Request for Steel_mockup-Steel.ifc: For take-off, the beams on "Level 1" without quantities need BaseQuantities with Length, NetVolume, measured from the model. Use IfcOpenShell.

First a look at what the model holds.

```python
import ifcopenshell
import ifcopenshell.util.element
import ifcopenshell.util.unit

model = ifcopenshell.open("Steel_mockup-Steel.ifc")
print(model.schema)
for unit_type in ("LENGTHUNIT", "AREAUNIT", "VOLUMEUNIT"):
    print(unit_type, ifcopenshell.util.unit.calculate_unit_scale(model, unit_type))
storey = next(s for s in model.by_type("IfcBuildingStorey") if s.Name == "Level 1")
beams = [e for e in ifcopenshell.util.element.get_decomposition(storey) if e.is_a("IfcBeam")]
for e in sorted(beams, key=lambda e: e.id()):
    print(e.id(), e.is_a(), e.Name, list(ifcopenshell.util.element.get_psets(e, qtos_only=True)), sep=" | ")
```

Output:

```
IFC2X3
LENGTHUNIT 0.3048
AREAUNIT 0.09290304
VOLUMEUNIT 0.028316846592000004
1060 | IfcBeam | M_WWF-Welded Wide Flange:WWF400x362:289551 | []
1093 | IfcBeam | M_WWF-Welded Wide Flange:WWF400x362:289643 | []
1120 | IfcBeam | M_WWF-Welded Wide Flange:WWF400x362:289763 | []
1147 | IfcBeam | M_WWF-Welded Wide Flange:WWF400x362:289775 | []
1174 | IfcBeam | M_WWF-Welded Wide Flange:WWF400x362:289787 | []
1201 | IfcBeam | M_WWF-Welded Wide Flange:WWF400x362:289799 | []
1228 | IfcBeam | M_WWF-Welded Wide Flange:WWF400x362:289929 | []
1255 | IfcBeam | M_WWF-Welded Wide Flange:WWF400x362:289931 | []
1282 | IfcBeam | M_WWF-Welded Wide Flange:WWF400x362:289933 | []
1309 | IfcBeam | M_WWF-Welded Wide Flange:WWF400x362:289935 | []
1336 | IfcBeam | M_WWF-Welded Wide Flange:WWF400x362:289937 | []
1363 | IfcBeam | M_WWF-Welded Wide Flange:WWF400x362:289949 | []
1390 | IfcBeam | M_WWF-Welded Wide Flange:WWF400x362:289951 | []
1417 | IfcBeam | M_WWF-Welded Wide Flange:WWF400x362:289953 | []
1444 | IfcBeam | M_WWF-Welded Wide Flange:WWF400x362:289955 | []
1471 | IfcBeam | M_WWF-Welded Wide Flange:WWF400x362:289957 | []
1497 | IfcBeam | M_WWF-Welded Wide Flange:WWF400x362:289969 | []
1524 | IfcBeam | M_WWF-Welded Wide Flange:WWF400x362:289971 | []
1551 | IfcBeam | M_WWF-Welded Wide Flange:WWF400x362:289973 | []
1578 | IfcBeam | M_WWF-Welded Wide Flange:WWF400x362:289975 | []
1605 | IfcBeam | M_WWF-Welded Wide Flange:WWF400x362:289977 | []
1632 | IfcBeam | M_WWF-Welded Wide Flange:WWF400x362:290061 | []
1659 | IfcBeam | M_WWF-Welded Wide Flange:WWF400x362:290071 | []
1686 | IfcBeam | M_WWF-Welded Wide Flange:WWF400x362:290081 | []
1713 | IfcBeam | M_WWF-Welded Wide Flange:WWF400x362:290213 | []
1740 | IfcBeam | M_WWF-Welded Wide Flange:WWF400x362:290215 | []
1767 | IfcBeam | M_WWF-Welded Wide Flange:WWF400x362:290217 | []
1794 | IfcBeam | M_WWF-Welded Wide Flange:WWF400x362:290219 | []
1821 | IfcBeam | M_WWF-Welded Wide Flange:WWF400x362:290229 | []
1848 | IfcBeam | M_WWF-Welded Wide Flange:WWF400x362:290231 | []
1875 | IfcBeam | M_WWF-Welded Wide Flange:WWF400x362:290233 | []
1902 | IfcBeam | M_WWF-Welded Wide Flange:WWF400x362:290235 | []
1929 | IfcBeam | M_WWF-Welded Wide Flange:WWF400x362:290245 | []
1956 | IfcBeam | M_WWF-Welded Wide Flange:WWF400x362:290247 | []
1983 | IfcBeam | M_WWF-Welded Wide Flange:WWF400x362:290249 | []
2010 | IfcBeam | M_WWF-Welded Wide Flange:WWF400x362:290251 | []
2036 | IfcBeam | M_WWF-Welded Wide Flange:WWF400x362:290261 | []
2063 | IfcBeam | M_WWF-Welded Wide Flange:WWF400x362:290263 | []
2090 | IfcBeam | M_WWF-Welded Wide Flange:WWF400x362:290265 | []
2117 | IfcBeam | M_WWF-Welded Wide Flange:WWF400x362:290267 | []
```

```python
import ifcopenshell
import ifcopenshell.api.pset
import ifcopenshell.geom
import ifcopenshell.util.element
import ifcopenshell.util.shape
import ifcopenshell.util.unit

model = ifcopenshell.open("Steel_mockup-Steel.ifc")
unit_scale = ifcopenshell.util.unit.calculate_unit_scale(model)
volume_scale = ifcopenshell.util.unit.calculate_unit_scale(model, "VOLUMEUNIT")
settings = ifcopenshell.geom.settings()

storey = next(s for s in model.by_type("IfcBuildingStorey") if s.Name == "Level 1")
beams = [e for e in ifcopenshell.util.element.get_decomposition(storey) if e.is_a("IfcBeam")]

for e in sorted(beams, key=lambda e: e.id()):
    if ifcopenshell.util.element.get_psets(e, qtos_only=True, should_inherit=False):
        continue
    # Geometry comes back in metres, in the element's own axes.
    shape = ifcopenshell.geom.create_shape(settings, e)
    values = {
        "Length": ifcopenshell.util.shape.get_max_xyz(shape.geometry) / unit_scale,
        "NetVolume": ifcopenshell.util.shape.get_volume(shape.geometry) / volume_scale,
    }
    qto = ifcopenshell.api.pset.add_qto(model, product=e, name="BaseQuantities")
    ifcopenshell.api.pset.edit_qto(model, qto=qto, properties=values)
    print(e.id(), {k: round(v, 3) for k, v in values.items()})

model.write("Steel_mockup-Steel_updated.ifc")
```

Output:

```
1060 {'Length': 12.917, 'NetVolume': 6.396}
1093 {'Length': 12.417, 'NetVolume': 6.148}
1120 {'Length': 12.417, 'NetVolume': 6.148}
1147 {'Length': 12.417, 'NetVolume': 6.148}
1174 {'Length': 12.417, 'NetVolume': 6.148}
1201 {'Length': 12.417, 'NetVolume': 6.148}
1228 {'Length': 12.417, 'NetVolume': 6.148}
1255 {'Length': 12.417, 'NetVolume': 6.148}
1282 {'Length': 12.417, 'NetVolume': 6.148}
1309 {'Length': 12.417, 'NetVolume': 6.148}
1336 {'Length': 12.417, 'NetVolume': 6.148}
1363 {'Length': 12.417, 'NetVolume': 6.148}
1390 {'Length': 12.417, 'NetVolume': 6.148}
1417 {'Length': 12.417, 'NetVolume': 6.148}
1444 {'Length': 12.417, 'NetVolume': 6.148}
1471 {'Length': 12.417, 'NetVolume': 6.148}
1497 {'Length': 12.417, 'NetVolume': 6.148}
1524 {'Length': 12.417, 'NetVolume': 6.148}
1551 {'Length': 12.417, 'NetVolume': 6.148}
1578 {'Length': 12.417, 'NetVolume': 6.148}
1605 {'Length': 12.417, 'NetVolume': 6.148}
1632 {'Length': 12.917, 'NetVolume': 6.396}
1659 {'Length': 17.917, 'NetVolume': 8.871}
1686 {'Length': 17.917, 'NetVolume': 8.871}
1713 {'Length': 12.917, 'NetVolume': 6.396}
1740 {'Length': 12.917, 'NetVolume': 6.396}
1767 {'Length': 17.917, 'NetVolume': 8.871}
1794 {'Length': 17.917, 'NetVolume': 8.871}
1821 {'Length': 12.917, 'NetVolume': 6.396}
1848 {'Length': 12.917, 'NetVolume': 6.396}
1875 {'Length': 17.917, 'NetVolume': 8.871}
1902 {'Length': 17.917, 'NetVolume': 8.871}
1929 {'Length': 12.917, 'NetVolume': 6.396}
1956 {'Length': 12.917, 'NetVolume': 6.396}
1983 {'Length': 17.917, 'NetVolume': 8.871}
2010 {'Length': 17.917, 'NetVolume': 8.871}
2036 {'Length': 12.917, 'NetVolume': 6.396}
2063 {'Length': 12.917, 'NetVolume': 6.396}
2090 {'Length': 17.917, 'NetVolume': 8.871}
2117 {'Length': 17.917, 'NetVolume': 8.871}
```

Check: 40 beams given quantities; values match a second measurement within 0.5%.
